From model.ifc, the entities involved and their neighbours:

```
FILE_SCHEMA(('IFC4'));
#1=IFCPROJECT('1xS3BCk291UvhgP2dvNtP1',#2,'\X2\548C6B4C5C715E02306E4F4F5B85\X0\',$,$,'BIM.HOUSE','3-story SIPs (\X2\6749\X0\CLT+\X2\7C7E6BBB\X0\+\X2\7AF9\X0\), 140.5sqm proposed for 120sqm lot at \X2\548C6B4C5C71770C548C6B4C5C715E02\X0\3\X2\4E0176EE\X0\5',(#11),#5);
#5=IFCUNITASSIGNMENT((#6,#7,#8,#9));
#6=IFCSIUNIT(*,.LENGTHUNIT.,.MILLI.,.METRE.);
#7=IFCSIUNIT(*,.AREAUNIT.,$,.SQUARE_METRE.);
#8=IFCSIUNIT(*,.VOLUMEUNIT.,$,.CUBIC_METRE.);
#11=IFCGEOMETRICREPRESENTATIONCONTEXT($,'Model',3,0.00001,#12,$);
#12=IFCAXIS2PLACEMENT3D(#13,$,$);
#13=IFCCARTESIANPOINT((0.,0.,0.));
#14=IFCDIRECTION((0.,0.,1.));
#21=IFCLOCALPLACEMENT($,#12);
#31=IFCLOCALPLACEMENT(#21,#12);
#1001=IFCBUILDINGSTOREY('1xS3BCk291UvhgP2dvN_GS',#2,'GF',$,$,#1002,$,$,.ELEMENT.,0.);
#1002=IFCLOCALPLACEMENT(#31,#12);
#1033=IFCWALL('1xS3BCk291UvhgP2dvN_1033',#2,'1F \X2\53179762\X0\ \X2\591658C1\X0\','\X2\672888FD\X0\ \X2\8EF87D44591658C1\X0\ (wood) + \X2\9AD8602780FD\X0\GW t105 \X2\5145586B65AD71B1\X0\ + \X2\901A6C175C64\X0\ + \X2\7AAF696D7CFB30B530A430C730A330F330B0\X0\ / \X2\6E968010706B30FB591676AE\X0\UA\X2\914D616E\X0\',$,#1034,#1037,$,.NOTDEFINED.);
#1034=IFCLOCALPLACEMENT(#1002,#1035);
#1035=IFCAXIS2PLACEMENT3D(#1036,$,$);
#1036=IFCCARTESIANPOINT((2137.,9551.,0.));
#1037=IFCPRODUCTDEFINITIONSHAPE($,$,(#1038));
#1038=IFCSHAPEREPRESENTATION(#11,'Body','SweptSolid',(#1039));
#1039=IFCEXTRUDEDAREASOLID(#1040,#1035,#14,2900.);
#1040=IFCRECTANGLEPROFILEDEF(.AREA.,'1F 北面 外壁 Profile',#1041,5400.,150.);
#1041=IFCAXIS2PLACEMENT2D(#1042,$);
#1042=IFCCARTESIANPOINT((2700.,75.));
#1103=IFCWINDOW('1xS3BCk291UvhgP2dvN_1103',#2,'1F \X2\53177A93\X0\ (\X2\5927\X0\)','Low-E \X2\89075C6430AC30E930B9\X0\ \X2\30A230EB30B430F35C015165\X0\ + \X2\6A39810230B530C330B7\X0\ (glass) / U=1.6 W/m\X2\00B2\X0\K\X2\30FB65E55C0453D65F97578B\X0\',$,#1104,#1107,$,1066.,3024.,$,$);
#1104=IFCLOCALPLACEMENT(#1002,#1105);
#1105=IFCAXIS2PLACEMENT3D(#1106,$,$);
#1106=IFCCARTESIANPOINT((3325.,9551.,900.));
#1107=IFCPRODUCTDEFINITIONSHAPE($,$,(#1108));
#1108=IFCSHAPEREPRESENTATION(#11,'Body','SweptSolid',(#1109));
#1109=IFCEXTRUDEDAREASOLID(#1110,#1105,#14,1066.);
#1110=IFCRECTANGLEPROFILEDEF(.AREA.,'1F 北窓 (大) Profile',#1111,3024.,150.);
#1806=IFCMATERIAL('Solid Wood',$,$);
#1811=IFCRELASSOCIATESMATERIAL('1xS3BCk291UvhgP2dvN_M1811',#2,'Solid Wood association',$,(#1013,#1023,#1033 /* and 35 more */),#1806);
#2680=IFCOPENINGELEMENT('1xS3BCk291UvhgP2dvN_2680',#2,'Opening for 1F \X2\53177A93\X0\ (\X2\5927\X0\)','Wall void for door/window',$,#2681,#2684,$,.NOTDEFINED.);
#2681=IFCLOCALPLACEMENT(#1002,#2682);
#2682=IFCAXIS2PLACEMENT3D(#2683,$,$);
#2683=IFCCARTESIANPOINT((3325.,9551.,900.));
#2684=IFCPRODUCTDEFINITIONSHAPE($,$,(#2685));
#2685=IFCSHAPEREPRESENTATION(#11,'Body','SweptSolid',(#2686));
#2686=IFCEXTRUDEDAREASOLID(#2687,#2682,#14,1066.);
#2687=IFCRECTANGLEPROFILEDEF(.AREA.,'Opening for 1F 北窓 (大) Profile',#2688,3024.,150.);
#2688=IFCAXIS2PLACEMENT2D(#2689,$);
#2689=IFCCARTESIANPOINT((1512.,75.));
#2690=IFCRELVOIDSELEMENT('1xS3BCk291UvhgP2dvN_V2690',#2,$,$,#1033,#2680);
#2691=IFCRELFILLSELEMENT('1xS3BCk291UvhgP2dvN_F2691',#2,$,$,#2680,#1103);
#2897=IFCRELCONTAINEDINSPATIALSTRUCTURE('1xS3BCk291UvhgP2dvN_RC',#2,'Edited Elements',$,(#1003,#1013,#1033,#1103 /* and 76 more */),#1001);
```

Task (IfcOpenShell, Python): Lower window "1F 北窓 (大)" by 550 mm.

```python
import numpy as np
import ifcopenshell
import ifcopenshell.api.geometry
import ifcopenshell.util.placement
import ifcopenshell.util.unit

model = ifcopenshell.open("model.ifc")
unit_scale = ifcopenshell.util.unit.calculate_unit_scale(model)

window = model.by_id(1103)
opening = window.FillsVoids[0].RelatingOpeningElement
dz = -550.0

shift = np.array([0.0, 0.0, dz])
# The window is not placed relative to its opening, so move both.
for product in (opening, window):
    matrix = ifcopenshell.util.placement.get_local_placement(product.ObjectPlacement)
    matrix[:3, 3] += shift
    ifcopenshell.api.geometry.edit_object_placement(model, product=product, matrix=matrix, is_si=False)

print(f"moved by {dz * unit_scale:+.3f} m")

model.write("model_rev.ifc")
```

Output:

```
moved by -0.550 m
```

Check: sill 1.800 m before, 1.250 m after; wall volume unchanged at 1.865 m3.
